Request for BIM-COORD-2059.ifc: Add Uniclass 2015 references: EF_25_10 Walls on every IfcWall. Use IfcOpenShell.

First a look at what the model holds.

```python
import ifcopenshell

model = ifcopenshell.open("BIM-COORD-2059.ifc")
print(model.schema)
print("classifications:", [c.Name for c in model.by_type("IfcClassification")])
for ifc_class in ("IfcDoor", "IfcRoof", "IfcStair", "IfcWall", "IfcWindow"):
    print(ifc_class, len(model.by_type(ifc_class)))
```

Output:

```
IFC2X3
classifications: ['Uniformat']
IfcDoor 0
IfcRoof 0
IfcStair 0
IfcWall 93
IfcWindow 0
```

```python
import ifcopenshell
import ifcopenshell.api.classification

model = ifcopenshell.open("BIM-COORD-2059.ifc")

# IFC2X3 requires Source and Edition and has no link from the project to the system.
system = model.create_entity("IfcClassification", Source="NBS", Edition="2015", Name="Uniclass 2015")

codes = {
    "IfcWall": ("EF_25_10", "Walls"),
}
for ifc_class, (code, name) in codes.items():
    products = model.by_type(ifc_class)
    ifcopenshell.api.classification.add_reference(
        model, products=products, classification=system, identification=code, name=name
    )
    print(code, len(products))

model.write("BIM-COORD-2059_rev.ifc")
```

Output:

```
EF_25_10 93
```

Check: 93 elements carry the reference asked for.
